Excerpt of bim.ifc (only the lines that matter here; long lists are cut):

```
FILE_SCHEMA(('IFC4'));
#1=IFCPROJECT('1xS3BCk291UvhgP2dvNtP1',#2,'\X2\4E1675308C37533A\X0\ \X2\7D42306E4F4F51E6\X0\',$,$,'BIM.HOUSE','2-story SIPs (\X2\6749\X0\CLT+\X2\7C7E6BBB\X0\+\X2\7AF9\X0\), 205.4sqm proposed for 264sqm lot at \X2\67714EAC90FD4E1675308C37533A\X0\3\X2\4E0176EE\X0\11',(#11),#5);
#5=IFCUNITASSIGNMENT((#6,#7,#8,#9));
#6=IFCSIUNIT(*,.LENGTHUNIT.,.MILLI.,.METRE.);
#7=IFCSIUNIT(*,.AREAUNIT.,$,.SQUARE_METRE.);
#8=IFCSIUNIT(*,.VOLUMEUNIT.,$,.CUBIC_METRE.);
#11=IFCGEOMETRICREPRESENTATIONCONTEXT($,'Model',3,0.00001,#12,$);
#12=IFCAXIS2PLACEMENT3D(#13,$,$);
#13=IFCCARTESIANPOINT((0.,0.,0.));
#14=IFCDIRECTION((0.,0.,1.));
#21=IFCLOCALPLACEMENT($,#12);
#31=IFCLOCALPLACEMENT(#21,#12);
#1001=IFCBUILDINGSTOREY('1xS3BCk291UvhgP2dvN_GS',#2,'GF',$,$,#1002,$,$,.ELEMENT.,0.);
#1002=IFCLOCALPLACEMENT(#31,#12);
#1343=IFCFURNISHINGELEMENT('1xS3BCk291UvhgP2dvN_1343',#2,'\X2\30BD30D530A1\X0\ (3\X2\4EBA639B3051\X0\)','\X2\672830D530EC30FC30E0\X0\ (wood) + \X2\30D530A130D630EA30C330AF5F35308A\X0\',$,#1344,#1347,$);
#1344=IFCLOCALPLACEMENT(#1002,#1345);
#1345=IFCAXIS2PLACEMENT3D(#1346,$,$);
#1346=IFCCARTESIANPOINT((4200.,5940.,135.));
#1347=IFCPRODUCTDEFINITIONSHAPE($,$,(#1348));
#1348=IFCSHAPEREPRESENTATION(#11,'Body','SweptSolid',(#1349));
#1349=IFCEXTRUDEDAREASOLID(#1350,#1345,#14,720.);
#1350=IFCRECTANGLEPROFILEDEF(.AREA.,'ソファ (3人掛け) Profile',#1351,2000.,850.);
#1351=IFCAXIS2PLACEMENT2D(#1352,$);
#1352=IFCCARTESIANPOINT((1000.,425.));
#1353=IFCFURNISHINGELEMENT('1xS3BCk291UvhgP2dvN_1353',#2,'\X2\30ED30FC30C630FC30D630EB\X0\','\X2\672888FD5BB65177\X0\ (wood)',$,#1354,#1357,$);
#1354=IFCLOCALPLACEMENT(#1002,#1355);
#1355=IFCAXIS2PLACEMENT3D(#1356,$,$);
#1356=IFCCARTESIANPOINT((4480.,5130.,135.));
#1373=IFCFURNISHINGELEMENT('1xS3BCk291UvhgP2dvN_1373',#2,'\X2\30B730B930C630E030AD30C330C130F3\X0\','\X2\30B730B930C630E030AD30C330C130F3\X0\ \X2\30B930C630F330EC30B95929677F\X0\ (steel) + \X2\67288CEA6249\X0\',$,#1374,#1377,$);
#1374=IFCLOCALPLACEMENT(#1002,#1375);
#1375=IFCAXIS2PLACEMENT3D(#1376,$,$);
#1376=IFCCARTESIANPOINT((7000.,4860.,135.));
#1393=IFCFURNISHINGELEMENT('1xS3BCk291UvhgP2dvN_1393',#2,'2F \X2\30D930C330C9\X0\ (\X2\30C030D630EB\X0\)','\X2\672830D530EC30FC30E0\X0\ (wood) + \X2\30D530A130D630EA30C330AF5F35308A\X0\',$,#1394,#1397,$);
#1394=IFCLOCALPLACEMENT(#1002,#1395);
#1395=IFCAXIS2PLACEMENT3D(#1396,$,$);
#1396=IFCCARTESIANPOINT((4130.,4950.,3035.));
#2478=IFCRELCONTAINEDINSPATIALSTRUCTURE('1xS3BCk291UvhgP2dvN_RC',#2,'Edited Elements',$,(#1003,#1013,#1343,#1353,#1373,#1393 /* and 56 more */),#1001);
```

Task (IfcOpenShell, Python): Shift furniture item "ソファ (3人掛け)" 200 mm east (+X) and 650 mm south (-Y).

```python
import ifcopenshell
import ifcopenshell.api.geometry
import ifcopenshell.util.placement
import ifcopenshell.util.unit

model = ifcopenshell.open("bim.ifc")
unit_scale = ifcopenshell.util.unit.calculate_unit_scale(model)

item = model.by_guid("1xS3BCk291UvhgP2dvN_1343")
matrix = ifcopenshell.util.placement.get_local_placement(item.ObjectPlacement)
matrix[0, 3] += 0.2 / unit_scale
matrix[1, 3] -= 0.65 / unit_scale
ifcopenshell.api.geometry.edit_object_placement(model, product=item, matrix=matrix, is_si=False)

print(ifcopenshell.util.placement.get_local_placement(item.ObjectPlacement).round(3) + 0.0)

model.write("bim_v2.ifc")
```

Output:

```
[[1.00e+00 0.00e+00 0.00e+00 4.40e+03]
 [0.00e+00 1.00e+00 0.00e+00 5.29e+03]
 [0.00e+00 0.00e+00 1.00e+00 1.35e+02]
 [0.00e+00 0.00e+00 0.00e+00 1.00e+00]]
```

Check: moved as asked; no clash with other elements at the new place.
